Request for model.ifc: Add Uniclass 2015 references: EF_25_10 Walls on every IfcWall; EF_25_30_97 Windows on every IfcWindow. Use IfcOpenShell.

First a look at what the model holds.

```python
import ifcopenshell

model = ifcopenshell.open("model.ifc")
print(model.schema)
print("classifications:", [c.Name for c in model.by_type("IfcClassification")])
for ifc_class in ("IfcDoor", "IfcRoof", "IfcStair", "IfcWall", "IfcWindow"):
    print(ifc_class, len(model.by_type(ifc_class)))
```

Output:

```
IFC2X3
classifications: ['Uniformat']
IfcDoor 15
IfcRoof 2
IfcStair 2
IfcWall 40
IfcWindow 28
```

```python
import ifcopenshell
import ifcopenshell.api.classification

model = ifcopenshell.open("model.ifc")

# IFC2X3 requires Source and Edition and has no link from the project to the system.
system = model.create_entity("IfcClassification", Source="NBS", Edition="2015", Name="Uniclass 2015")

codes = {
    "IfcWall": ("EF_25_10", "Walls"),
    "IfcWindow": ("EF_25_30_97", "Windows"),
}
for ifc_class, (code, name) in codes.items():
    products = model.by_type(ifc_class)
    ifcopenshell.api.classification.add_reference(
        model, products=products, classification=system, identification=code, name=name
    )
    print(code, len(products))

model.write("model-out.ifc")
```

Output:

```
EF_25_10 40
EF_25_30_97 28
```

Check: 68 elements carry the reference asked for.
